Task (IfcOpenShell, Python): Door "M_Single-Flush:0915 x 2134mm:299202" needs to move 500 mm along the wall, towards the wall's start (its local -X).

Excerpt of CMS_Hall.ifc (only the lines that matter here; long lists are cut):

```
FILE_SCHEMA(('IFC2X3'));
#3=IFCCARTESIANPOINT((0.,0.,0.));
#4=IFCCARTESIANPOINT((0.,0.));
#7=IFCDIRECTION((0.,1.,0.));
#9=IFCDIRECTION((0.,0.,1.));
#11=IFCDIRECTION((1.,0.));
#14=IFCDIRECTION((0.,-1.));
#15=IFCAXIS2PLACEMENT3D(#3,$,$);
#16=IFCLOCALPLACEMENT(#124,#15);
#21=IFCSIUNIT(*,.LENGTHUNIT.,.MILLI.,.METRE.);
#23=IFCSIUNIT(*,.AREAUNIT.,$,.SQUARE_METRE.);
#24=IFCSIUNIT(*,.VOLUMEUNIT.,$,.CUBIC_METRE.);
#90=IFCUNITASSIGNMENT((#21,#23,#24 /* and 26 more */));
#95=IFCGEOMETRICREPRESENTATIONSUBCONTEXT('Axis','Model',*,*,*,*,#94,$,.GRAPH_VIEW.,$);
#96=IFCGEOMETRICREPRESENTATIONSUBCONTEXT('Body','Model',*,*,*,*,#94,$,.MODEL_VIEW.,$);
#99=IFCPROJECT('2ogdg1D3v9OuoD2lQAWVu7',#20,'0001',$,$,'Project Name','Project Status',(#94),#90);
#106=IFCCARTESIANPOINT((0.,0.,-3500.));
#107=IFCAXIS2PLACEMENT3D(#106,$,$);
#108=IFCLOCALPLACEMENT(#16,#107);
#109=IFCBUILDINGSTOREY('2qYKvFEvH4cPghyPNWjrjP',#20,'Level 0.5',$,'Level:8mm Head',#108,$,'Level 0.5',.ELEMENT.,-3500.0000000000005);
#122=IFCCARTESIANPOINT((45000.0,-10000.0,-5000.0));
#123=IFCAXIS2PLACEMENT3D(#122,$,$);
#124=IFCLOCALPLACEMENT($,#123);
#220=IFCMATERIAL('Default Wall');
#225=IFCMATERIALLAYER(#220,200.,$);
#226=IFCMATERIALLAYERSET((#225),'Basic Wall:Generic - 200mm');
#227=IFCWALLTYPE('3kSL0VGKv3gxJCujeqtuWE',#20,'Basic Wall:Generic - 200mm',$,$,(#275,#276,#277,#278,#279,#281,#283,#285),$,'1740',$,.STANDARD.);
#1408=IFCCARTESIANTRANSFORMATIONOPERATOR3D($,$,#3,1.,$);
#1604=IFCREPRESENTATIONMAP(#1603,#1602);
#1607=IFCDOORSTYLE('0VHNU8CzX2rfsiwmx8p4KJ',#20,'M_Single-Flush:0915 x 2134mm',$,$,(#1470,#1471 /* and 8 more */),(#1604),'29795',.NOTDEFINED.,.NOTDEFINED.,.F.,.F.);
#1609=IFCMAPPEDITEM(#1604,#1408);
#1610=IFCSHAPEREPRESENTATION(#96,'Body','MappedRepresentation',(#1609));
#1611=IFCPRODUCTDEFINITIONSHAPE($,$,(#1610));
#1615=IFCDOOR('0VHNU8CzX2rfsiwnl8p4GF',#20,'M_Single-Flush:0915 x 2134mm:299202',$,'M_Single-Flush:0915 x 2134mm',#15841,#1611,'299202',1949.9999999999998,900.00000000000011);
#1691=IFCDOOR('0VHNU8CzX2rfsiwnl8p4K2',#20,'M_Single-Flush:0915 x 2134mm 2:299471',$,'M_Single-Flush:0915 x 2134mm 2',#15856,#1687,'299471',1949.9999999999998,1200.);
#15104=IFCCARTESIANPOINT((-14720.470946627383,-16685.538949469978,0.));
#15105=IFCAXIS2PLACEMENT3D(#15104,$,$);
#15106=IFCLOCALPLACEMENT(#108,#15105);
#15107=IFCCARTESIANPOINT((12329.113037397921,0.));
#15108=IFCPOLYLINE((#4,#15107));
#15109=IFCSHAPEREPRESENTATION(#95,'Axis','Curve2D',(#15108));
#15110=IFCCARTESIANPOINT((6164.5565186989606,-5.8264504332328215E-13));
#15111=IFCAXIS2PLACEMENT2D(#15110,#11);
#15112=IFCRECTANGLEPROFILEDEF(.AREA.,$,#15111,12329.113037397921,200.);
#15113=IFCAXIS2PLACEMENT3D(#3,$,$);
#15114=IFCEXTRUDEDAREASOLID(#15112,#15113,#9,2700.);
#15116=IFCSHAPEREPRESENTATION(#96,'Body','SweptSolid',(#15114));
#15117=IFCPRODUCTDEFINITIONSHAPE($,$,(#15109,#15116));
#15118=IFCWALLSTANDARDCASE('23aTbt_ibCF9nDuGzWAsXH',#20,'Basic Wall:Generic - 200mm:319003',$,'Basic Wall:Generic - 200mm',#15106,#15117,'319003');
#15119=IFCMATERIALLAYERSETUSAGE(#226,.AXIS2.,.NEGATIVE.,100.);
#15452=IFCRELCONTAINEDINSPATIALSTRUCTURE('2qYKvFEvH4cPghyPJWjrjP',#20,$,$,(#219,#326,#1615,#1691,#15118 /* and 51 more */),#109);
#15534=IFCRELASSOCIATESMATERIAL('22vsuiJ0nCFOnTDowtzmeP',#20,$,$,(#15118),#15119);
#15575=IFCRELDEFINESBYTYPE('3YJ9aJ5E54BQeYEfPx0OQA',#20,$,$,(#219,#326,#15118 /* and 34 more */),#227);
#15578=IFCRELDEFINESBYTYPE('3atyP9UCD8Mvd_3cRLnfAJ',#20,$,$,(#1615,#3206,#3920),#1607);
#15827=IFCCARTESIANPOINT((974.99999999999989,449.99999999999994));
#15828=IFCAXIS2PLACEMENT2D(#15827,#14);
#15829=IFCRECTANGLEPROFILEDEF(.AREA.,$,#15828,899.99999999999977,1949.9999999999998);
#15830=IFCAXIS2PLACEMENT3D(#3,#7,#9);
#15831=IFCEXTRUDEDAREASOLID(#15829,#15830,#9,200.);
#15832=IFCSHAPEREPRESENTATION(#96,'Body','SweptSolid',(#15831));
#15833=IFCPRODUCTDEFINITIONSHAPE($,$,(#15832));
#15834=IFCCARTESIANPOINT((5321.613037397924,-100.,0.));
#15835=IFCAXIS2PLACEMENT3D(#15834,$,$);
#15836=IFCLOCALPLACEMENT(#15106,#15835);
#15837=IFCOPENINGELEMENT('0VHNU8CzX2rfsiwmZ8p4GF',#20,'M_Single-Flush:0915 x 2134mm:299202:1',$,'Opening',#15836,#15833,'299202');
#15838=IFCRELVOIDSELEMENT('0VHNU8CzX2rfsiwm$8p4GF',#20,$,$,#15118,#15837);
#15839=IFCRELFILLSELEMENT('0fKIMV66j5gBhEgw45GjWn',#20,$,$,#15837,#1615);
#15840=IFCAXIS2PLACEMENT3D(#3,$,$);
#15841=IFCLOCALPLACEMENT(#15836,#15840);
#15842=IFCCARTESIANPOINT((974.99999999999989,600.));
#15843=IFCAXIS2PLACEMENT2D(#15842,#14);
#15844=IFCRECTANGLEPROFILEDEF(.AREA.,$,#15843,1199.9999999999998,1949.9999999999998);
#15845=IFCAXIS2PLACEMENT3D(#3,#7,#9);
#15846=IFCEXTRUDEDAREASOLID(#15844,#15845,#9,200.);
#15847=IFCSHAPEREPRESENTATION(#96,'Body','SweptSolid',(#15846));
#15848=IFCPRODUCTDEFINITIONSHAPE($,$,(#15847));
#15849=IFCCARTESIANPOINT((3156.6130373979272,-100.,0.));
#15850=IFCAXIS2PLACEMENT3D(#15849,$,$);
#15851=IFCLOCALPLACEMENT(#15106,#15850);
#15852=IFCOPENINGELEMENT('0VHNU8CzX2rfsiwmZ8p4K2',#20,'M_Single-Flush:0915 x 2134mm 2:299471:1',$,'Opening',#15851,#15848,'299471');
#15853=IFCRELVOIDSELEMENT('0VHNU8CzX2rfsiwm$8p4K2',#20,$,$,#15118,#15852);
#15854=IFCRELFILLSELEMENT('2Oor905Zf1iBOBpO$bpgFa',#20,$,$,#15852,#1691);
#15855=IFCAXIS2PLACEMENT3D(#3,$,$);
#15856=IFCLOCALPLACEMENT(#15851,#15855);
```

```python
import ifcopenshell
import ifcopenshell.api.geometry
import ifcopenshell.util.placement
import ifcopenshell.util.unit

model = ifcopenshell.open("CMS_Hall.ifc")
unit_scale = ifcopenshell.util.unit.calculate_unit_scale(model)

door = model.by_guid("0VHNU8CzX2rfsiwnl8p4GF")
opening = door.FillsVoids[0].RelatingOpeningElement
wall = opening.VoidsElements[0].RelatingBuildingElement

wall_matrix = ifcopenshell.util.placement.get_local_placement(wall.ObjectPlacement)
shift = wall_matrix[:3, 0] * -0.5 / unit_scale
before = ifcopenshell.util.placement.get_local_placement(door.ObjectPlacement)[:3, 3].copy()

# The door is placed relative to its opening, so it follows when the opening moves.
matrix = ifcopenshell.util.placement.get_local_placement(opening.ObjectPlacement)
matrix[:3, 3] += shift
ifcopenshell.api.geometry.edit_object_placement(
    model, product=opening, matrix=matrix, is_si=False, should_transform_children=True
)

after = ifcopenshell.util.placement.get_local_placement(door.ObjectPlacement)[:3, 3]
print("door moved by", (after - before).round(3) + 0.0)

model.write("CMS_Hall_rev.ifc")
```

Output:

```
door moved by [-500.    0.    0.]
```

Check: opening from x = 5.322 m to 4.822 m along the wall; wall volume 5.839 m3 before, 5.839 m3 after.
